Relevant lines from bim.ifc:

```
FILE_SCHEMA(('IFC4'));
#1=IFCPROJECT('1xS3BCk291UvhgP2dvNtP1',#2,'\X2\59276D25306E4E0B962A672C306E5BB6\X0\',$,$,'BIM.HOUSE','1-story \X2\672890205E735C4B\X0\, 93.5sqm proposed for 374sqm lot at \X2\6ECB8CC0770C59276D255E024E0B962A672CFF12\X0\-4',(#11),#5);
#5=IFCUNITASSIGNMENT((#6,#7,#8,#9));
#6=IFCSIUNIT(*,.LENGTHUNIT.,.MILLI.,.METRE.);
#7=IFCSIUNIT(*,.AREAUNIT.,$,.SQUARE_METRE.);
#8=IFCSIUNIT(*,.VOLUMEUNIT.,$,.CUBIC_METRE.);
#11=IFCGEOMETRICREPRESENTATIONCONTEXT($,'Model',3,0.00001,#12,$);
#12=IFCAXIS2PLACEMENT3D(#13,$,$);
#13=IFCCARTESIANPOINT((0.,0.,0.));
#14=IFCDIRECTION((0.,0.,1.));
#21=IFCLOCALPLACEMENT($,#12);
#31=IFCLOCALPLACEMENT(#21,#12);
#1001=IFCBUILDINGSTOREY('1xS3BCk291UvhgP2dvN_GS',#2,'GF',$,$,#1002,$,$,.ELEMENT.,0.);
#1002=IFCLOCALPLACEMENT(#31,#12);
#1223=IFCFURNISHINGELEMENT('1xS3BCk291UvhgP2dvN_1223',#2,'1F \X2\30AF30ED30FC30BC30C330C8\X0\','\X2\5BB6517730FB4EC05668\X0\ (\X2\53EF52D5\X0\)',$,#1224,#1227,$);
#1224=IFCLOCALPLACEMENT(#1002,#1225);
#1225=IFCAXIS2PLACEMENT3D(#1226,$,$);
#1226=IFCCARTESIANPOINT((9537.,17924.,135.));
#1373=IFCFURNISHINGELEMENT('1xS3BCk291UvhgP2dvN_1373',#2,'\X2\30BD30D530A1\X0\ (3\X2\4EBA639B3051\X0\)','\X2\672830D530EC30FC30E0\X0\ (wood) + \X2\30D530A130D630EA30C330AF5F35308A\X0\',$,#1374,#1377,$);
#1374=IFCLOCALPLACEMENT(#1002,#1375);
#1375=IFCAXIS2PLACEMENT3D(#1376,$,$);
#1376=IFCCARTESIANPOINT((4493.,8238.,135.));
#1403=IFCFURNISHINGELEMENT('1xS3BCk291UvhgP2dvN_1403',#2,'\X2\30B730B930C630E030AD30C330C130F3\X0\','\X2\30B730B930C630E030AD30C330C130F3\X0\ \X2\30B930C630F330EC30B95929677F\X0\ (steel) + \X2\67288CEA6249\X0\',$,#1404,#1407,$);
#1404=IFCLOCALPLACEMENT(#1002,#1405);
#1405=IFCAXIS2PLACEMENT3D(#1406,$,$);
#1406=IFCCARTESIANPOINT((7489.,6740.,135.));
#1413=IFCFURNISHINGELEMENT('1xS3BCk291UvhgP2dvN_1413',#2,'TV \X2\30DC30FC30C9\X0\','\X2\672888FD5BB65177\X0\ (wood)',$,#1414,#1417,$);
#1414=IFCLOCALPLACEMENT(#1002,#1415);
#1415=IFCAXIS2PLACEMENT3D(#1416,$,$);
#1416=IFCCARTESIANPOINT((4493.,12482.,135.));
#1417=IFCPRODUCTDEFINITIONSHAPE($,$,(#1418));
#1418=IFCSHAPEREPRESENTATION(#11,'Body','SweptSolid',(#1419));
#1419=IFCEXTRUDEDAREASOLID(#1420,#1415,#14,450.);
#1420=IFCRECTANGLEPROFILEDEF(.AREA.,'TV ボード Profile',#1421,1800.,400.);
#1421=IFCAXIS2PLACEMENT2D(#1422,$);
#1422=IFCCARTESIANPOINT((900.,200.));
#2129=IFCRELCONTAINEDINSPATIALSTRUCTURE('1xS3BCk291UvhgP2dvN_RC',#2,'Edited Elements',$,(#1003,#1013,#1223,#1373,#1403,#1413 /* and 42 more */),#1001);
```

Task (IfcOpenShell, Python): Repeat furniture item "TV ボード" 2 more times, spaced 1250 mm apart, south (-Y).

```python
import numpy as np
import ifcopenshell
import ifcopenshell.api.geometry
import ifcopenshell.api.root
import ifcopenshell.util.element
import ifcopenshell.util.placement
import ifcopenshell.util.unit

model = ifcopenshell.open("bim.ifc")
unit_scale = ifcopenshell.util.unit.calculate_unit_scale(model)


def reuse_history(source, copy):
    """copy_class also copies each property set's owner history, people and application; keep the originals."""
    for rel in copy.IsDefinedBy:
        if rel.is_a("IfcRelDefinesByProperties") and (history := rel.RelatingPropertyDefinition.OwnerHistory):
            rel.RelatingPropertyDefinition.OwnerHistory = source.OwnerHistory
            ifcopenshell.util.element.remove_deep2(model, history)


source = model.by_guid("1xS3BCk291UvhgP2dvN_1413")
base = ifcopenshell.util.placement.get_local_placement(source.ObjectPlacement)
step = np.array([0.0, -1.0, 0.0]) * 1.25 / unit_scale

for i in range(1, 3):
    copy = ifcopenshell.api.root.copy_class(model, product=source)
    copy.Representation = ifcopenshell.util.element.copy_deep(
        model, source.Representation, exclude=["IfcGeometricRepresentationContext", "IfcRepresentationMap"]
    )
    reuse_history(source, copy)
    matrix = base.copy()
    matrix[:3, 3] += i * step
    print("added at", matrix[:3, 3].round(3) + 0.0)
    ifcopenshell.api.geometry.edit_object_placement(model, product=copy, matrix=matrix, is_si=False)

model.write("bim_updated.ifc")
```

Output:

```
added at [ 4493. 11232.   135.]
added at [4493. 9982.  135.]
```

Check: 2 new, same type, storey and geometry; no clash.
